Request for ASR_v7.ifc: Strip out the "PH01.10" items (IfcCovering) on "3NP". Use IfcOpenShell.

First a look at what the model holds.

```python
import ifcopenshell
import ifcopenshell.util.element

model = ifcopenshell.open("ASR_v7.ifc")
print(model.schema)
storey = next(s for s in model.by_type("IfcBuildingStorey") if s.Name == "3NP")
coverings = [e for e in ifcopenshell.util.element.get_decomposition(storey) if e.is_a("IfcCovering")]
seen = {}
for e in coverings:
    element_type = ifcopenshell.util.element.get_type(e)
    name = element_type.Name if element_type not in (None, e) else None
    seen[name] = seen.get(name, 0) + 1
for name, count in sorted(seen.items(), key=str):
    print(count, "x", name)
```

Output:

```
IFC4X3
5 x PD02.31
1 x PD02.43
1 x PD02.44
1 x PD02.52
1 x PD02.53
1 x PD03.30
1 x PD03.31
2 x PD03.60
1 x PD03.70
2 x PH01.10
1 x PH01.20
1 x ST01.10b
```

```python
import ifcopenshell
import ifcopenshell.api.root
import ifcopenshell.util.element

model = ifcopenshell.open("ASR_v7.ifc")

storey = next(s for s in model.by_type("IfcBuildingStorey") if s.Name == "3NP")
coverings = [e for e in ifcopenshell.util.element.get_decomposition(storey) if e.is_a("IfcCovering")]
targets = [e for e in coverings if (t := ifcopenshell.util.element.get_type(e)) not in (None, e) and t.Name == "PH01.10"]

for e in targets:
    ifcopenshell.api.root.remove_product(model, product=e)
print(len(targets), "removed")

model.write("ASR_v7-out.ifc")
```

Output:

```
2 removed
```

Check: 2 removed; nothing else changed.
